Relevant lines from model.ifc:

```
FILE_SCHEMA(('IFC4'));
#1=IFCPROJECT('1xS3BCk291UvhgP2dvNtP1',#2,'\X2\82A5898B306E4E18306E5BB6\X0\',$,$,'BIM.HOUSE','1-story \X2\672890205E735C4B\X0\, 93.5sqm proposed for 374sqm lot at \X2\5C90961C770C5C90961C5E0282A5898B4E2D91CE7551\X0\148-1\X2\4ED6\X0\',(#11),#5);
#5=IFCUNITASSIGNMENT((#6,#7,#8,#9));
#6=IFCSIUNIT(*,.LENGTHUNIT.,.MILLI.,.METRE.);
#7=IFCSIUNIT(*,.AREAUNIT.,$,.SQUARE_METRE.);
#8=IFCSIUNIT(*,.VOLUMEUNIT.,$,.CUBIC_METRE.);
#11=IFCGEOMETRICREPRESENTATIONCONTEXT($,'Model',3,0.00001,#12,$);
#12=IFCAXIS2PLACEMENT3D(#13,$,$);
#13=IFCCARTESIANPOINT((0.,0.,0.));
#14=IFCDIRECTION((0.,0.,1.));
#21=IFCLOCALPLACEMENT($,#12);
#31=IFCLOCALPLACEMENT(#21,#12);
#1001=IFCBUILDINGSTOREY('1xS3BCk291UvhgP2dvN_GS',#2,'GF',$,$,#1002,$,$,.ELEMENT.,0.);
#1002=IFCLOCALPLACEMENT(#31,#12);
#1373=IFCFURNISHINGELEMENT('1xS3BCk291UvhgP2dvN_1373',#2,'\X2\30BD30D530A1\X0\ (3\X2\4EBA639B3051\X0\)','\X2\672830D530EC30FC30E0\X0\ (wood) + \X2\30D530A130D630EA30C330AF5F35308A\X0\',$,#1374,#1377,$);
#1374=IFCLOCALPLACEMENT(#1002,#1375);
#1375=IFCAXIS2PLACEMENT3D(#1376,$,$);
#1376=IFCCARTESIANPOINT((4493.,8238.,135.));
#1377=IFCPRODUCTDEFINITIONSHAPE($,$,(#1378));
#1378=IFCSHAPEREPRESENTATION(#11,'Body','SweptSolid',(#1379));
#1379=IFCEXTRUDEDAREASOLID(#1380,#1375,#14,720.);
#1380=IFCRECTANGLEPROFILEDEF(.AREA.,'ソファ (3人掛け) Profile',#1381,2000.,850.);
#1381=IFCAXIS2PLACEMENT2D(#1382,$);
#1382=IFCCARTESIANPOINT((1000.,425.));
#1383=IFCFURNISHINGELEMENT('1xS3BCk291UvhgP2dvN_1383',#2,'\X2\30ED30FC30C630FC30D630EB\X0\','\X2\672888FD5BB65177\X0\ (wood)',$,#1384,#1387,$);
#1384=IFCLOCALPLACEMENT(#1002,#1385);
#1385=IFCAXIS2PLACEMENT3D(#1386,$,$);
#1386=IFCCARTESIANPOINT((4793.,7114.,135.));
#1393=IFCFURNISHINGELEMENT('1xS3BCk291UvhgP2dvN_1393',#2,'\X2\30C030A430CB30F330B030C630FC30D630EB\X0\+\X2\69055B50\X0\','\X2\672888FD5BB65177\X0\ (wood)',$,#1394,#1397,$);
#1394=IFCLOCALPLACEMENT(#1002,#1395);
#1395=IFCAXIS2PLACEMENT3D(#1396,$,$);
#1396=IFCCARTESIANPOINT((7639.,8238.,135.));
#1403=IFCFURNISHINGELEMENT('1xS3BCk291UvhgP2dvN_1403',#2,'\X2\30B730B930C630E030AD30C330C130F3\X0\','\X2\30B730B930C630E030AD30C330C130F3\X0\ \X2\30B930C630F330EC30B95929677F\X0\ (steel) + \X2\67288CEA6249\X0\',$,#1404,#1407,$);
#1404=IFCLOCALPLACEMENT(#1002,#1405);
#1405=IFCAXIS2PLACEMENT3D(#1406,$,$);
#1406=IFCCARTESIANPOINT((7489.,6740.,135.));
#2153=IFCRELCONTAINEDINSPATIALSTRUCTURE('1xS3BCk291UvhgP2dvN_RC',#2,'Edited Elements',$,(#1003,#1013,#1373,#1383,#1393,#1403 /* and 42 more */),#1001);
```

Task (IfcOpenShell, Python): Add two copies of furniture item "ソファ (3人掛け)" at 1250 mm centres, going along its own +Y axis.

```python
import ifcopenshell
import ifcopenshell.api.geometry
import ifcopenshell.api.root
import ifcopenshell.util.element
import ifcopenshell.util.placement
import ifcopenshell.util.unit

model = ifcopenshell.open("model.ifc")
unit_scale = ifcopenshell.util.unit.calculate_unit_scale(model)


def reuse_history(source, copy):
    """copy_class also copies each property set's owner history, people and application; keep the originals."""
    for rel in copy.IsDefinedBy:
        if rel.is_a("IfcRelDefinesByProperties") and (history := rel.RelatingPropertyDefinition.OwnerHistory):
            rel.RelatingPropertyDefinition.OwnerHistory = source.OwnerHistory
            ifcopenshell.util.element.remove_deep2(model, history)


source = model.by_guid("1xS3BCk291UvhgP2dvN_1373")
base = ifcopenshell.util.placement.get_local_placement(source.ObjectPlacement)
step = base[:3, 1] * 1.25 / unit_scale

for i in range(1, 3):
    copy = ifcopenshell.api.root.copy_class(model, product=source)
    copy.Representation = ifcopenshell.util.element.copy_deep(
        model, source.Representation, exclude=["IfcGeometricRepresentationContext", "IfcRepresentationMap"]
    )
    reuse_history(source, copy)
    matrix = base.copy()
    matrix[:3, 3] += i * step
    print("added at", matrix[:3, 3].round(3) + 0.0)
    ifcopenshell.api.geometry.edit_object_placement(model, product=copy, matrix=matrix, is_si=False)

model.write("model_edited.ifc")
```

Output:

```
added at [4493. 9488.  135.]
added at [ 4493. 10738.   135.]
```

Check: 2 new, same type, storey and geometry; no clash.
